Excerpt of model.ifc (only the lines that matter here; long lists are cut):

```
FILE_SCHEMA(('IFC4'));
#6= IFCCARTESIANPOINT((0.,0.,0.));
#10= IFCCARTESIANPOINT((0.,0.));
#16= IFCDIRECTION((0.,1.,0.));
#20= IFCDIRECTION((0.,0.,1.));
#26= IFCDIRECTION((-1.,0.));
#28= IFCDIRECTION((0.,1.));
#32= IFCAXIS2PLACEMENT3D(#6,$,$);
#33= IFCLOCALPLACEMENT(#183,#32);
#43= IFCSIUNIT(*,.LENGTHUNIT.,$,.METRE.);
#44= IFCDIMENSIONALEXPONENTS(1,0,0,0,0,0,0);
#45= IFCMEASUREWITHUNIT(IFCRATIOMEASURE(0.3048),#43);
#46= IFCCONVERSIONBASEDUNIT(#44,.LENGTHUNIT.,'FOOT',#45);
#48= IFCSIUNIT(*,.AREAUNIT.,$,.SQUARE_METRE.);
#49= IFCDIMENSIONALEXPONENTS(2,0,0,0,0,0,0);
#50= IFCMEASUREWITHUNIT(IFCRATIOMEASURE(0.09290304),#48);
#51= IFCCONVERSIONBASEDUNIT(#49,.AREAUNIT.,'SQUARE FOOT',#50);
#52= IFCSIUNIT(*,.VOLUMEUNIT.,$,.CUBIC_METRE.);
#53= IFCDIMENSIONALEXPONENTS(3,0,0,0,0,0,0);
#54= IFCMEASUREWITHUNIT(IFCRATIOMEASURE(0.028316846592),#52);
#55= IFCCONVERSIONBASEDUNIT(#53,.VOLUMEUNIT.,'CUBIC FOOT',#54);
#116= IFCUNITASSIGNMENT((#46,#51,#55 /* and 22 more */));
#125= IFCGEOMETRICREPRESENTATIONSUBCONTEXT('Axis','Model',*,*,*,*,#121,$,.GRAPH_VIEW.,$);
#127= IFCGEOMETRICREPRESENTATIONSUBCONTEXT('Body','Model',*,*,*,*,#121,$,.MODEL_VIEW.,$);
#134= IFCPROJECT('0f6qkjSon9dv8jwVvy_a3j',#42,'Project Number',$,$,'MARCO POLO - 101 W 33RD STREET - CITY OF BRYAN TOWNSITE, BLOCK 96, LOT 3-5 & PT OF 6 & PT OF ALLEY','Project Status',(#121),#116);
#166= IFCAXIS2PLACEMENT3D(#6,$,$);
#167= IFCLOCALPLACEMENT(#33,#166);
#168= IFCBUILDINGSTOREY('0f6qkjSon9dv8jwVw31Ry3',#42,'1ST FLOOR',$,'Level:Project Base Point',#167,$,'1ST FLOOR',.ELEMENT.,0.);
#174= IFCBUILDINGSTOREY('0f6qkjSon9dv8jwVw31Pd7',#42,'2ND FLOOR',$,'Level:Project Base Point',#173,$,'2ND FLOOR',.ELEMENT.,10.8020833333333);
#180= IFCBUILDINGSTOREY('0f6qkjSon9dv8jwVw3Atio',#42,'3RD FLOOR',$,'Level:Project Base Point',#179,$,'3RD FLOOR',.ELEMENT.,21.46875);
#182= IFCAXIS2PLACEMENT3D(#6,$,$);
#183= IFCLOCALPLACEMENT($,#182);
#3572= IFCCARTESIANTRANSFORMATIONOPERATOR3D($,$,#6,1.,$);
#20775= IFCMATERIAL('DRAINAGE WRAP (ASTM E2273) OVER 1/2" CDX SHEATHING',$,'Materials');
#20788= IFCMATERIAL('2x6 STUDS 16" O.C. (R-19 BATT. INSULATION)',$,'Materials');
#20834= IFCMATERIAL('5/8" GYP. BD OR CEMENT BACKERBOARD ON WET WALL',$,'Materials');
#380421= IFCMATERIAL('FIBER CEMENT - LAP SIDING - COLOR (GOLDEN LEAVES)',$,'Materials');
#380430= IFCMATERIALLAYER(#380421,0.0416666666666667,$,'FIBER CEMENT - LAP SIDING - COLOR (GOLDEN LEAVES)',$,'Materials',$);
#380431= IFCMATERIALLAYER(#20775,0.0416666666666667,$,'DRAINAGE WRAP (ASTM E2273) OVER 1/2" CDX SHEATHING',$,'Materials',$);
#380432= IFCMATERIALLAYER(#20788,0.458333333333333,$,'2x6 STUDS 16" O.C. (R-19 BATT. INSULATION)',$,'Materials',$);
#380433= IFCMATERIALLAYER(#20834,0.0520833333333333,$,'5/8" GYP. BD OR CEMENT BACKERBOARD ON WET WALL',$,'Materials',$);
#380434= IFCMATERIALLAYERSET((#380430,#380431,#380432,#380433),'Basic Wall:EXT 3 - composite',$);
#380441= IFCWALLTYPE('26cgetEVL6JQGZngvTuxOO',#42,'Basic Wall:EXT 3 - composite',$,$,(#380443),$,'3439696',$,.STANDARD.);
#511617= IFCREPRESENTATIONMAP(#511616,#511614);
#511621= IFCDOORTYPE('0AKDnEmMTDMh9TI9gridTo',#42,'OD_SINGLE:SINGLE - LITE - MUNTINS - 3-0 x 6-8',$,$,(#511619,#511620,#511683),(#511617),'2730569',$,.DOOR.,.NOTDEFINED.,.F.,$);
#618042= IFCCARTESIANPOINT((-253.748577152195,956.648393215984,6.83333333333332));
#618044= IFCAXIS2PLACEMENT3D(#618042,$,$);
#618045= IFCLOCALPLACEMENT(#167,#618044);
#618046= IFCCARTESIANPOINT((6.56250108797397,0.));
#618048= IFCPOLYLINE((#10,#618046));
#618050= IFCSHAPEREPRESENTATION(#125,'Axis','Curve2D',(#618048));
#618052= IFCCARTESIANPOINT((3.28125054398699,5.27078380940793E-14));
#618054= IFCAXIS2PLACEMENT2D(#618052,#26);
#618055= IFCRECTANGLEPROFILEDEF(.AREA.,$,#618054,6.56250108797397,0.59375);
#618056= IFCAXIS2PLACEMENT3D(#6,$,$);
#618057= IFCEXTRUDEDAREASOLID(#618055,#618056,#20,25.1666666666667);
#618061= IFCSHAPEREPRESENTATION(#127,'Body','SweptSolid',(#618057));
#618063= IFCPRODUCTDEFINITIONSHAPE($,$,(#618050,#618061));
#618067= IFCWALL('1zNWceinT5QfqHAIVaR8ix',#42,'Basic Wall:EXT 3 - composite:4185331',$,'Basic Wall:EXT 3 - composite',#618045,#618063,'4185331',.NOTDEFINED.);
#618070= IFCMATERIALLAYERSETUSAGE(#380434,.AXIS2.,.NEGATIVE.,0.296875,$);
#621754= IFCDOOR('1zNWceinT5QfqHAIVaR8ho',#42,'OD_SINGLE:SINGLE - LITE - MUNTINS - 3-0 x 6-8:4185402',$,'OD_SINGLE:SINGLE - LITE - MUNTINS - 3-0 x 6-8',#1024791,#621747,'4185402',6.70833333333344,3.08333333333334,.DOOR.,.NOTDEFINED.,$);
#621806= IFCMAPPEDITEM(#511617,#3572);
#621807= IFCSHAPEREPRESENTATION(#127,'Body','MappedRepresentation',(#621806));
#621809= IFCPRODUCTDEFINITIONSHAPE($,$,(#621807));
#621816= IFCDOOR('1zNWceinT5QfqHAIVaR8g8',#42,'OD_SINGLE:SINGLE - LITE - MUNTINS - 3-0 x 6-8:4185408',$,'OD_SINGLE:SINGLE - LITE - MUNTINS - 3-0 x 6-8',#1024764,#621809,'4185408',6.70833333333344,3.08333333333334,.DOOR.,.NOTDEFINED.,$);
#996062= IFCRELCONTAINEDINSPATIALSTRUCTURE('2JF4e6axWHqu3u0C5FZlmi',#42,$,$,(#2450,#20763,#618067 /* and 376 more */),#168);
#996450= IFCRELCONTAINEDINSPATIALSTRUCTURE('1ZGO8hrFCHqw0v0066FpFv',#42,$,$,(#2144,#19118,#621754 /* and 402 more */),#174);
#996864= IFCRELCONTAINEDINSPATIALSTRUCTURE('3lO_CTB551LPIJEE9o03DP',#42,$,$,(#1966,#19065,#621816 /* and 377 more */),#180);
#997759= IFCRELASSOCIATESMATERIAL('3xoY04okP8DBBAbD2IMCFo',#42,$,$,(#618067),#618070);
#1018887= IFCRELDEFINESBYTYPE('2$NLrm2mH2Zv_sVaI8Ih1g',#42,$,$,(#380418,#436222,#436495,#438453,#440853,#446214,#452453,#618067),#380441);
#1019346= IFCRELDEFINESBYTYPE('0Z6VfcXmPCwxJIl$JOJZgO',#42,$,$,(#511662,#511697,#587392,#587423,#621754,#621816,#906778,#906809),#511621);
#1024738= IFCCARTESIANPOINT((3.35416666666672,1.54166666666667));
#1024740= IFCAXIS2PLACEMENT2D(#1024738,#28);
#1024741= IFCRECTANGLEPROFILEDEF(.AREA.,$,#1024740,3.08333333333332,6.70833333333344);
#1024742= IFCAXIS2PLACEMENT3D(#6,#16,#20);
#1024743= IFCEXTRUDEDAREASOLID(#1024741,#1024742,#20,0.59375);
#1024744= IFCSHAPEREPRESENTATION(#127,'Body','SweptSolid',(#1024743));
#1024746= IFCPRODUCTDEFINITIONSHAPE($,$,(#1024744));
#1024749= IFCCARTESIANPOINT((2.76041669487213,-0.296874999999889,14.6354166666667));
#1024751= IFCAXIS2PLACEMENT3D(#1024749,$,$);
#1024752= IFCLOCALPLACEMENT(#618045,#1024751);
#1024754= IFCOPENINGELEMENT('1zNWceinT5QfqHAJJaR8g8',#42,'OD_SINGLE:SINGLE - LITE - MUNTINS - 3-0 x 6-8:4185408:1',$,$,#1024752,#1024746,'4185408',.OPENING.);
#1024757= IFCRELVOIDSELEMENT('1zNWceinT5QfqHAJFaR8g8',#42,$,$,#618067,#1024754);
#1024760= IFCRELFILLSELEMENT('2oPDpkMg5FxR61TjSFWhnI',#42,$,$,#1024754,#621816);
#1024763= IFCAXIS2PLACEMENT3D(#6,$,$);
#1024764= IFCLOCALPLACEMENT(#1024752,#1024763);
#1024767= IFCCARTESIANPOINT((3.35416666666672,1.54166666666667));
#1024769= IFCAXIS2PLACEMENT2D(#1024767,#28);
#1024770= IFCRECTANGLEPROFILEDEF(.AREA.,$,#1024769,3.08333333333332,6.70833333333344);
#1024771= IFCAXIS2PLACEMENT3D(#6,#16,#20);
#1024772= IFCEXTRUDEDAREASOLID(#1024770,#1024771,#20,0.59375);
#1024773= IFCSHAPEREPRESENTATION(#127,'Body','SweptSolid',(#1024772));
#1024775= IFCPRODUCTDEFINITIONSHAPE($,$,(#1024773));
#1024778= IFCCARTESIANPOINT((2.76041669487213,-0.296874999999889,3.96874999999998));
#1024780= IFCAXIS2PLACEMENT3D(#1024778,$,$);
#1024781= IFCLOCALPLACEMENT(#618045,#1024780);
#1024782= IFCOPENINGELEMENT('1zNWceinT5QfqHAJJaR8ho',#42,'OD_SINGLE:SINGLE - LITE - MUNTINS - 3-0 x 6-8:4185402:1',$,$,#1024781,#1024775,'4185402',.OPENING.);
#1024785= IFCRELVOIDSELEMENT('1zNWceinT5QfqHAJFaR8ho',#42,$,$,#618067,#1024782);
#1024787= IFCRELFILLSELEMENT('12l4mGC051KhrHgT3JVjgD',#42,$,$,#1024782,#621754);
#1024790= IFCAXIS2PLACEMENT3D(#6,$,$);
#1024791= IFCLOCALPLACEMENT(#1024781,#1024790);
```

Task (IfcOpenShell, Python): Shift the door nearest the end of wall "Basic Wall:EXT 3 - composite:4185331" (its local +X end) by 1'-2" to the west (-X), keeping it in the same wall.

```python
import ifcopenshell
import ifcopenshell.api.geometry
import ifcopenshell.util.placement
import ifcopenshell.util.unit

model = ifcopenshell.open("model.ifc")
unit_scale = ifcopenshell.util.unit.calculate_unit_scale(model)

door = model.by_id(621816)
opening = door.FillsVoids[0].RelatingOpeningElement
wall = opening.VoidsElements[0].RelatingBuildingElement

wall_matrix = ifcopenshell.util.placement.get_local_placement(wall.ObjectPlacement)
shift = wall_matrix[:3, 0] * -14 * 0.0254 / unit_scale
before = ifcopenshell.util.placement.get_local_placement(door.ObjectPlacement)[:3, 3].copy()

# The door is placed relative to its opening, so it follows when the opening moves.
matrix = ifcopenshell.util.placement.get_local_placement(opening.ObjectPlacement)
matrix[:3, 3] += shift
ifcopenshell.api.geometry.edit_object_placement(
    model, product=opening, matrix=matrix, is_si=False, should_transform_children=True
)

after = ifcopenshell.util.placement.get_local_placement(door.ObjectPlacement)[:3, 3]
print("door moved by", (after - before).round(3) + 0.0)

model.write("model_edited.ifc")
```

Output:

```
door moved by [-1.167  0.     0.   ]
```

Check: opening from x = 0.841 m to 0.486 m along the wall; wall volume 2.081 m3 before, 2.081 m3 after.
